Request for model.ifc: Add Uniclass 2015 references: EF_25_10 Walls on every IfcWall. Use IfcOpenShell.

First a look at what the model holds.

```python
import ifcopenshell

model = ifcopenshell.open("model.ifc")
print(model.schema)
print("classifications:", [c.Name for c in model.by_type("IfcClassification")])
for ifc_class in ("IfcDoor", "IfcRoof", "IfcStair", "IfcWall", "IfcWindow"):
    print(ifc_class, len(model.by_type(ifc_class)))
```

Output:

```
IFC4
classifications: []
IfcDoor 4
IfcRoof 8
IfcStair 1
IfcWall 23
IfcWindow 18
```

```python
import ifcopenshell
import ifcopenshell.api.classification

model = ifcopenshell.open("model.ifc")

system = ifcopenshell.api.classification.add_classification(model, classification="Uniclass 2015")

codes = {
    "IfcWall": ("EF_25_10", "Walls"),
}
for ifc_class, (code, name) in codes.items():
    products = model.by_type(ifc_class)
    ifcopenshell.api.classification.add_reference(
        model, products=products, classification=system, identification=code, name=name
    )
    print(code, len(products))

model.write("model_edited.ifc")
```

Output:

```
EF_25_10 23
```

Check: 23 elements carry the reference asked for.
